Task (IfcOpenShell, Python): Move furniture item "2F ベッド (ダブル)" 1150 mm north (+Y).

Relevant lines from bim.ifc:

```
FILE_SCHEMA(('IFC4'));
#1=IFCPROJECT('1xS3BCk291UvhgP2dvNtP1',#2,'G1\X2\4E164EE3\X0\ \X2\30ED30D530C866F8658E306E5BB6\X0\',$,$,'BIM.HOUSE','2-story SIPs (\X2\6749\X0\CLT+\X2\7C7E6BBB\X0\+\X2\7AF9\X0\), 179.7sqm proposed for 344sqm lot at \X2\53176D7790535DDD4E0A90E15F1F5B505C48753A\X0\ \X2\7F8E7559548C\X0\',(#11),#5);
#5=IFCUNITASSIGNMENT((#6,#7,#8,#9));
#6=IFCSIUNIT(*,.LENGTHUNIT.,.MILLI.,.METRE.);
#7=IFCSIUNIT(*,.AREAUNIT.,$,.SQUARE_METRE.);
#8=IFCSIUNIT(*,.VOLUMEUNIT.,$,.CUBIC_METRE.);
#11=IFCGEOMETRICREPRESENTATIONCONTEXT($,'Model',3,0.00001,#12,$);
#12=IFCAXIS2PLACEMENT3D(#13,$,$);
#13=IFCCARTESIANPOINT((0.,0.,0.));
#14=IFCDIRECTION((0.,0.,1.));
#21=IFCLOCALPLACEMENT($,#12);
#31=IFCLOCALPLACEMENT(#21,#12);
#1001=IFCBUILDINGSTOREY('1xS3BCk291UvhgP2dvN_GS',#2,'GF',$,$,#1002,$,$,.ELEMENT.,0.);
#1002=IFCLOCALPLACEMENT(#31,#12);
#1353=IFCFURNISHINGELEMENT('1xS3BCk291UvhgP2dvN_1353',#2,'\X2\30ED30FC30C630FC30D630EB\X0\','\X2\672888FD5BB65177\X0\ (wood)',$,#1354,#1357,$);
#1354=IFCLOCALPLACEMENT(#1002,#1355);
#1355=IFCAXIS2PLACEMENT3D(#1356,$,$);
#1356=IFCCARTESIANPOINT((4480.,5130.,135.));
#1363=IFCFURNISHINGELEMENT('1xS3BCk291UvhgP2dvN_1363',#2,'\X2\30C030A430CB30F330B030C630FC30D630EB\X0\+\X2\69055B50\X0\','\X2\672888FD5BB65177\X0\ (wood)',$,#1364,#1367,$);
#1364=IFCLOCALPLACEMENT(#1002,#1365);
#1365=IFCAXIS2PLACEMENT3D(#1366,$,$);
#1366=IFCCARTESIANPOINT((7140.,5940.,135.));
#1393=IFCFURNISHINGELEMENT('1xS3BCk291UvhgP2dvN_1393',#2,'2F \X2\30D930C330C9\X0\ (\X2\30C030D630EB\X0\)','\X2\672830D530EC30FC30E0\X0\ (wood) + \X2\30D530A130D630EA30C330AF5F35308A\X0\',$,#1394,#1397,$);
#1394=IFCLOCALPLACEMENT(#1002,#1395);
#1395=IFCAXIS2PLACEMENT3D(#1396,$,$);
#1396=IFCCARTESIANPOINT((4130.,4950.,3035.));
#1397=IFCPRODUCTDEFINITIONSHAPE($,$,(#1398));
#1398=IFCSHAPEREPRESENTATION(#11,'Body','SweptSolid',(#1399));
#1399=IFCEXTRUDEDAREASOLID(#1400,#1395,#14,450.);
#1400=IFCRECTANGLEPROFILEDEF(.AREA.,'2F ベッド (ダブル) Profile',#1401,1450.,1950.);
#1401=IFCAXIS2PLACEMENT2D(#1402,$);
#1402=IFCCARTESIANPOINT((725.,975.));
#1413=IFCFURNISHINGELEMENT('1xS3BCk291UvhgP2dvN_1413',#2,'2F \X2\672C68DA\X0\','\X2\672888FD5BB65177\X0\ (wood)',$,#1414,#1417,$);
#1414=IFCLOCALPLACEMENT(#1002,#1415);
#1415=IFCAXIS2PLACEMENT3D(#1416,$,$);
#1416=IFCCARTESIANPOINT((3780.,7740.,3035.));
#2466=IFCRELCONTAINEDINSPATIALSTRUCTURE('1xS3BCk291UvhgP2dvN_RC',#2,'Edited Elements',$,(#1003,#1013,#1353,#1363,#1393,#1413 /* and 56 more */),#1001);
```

```python
import ifcopenshell
import ifcopenshell.api.geometry
import ifcopenshell.util.placement
import ifcopenshell.util.unit

model = ifcopenshell.open("bim.ifc")
unit_scale = ifcopenshell.util.unit.calculate_unit_scale(model)

item = model.by_guid("1xS3BCk291UvhgP2dvN_1393")
matrix = ifcopenshell.util.placement.get_local_placement(item.ObjectPlacement)
matrix[1, 3] += 1.15 / unit_scale
ifcopenshell.api.geometry.edit_object_placement(model, product=item, matrix=matrix, is_si=False)

print(ifcopenshell.util.placement.get_local_placement(item.ObjectPlacement).round(3) + 0.0)

model.write("bim_updated.ifc")
```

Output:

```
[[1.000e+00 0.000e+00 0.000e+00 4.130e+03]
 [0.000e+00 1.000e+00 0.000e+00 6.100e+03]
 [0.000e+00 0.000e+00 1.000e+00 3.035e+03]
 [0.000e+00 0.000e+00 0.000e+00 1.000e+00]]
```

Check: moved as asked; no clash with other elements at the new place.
